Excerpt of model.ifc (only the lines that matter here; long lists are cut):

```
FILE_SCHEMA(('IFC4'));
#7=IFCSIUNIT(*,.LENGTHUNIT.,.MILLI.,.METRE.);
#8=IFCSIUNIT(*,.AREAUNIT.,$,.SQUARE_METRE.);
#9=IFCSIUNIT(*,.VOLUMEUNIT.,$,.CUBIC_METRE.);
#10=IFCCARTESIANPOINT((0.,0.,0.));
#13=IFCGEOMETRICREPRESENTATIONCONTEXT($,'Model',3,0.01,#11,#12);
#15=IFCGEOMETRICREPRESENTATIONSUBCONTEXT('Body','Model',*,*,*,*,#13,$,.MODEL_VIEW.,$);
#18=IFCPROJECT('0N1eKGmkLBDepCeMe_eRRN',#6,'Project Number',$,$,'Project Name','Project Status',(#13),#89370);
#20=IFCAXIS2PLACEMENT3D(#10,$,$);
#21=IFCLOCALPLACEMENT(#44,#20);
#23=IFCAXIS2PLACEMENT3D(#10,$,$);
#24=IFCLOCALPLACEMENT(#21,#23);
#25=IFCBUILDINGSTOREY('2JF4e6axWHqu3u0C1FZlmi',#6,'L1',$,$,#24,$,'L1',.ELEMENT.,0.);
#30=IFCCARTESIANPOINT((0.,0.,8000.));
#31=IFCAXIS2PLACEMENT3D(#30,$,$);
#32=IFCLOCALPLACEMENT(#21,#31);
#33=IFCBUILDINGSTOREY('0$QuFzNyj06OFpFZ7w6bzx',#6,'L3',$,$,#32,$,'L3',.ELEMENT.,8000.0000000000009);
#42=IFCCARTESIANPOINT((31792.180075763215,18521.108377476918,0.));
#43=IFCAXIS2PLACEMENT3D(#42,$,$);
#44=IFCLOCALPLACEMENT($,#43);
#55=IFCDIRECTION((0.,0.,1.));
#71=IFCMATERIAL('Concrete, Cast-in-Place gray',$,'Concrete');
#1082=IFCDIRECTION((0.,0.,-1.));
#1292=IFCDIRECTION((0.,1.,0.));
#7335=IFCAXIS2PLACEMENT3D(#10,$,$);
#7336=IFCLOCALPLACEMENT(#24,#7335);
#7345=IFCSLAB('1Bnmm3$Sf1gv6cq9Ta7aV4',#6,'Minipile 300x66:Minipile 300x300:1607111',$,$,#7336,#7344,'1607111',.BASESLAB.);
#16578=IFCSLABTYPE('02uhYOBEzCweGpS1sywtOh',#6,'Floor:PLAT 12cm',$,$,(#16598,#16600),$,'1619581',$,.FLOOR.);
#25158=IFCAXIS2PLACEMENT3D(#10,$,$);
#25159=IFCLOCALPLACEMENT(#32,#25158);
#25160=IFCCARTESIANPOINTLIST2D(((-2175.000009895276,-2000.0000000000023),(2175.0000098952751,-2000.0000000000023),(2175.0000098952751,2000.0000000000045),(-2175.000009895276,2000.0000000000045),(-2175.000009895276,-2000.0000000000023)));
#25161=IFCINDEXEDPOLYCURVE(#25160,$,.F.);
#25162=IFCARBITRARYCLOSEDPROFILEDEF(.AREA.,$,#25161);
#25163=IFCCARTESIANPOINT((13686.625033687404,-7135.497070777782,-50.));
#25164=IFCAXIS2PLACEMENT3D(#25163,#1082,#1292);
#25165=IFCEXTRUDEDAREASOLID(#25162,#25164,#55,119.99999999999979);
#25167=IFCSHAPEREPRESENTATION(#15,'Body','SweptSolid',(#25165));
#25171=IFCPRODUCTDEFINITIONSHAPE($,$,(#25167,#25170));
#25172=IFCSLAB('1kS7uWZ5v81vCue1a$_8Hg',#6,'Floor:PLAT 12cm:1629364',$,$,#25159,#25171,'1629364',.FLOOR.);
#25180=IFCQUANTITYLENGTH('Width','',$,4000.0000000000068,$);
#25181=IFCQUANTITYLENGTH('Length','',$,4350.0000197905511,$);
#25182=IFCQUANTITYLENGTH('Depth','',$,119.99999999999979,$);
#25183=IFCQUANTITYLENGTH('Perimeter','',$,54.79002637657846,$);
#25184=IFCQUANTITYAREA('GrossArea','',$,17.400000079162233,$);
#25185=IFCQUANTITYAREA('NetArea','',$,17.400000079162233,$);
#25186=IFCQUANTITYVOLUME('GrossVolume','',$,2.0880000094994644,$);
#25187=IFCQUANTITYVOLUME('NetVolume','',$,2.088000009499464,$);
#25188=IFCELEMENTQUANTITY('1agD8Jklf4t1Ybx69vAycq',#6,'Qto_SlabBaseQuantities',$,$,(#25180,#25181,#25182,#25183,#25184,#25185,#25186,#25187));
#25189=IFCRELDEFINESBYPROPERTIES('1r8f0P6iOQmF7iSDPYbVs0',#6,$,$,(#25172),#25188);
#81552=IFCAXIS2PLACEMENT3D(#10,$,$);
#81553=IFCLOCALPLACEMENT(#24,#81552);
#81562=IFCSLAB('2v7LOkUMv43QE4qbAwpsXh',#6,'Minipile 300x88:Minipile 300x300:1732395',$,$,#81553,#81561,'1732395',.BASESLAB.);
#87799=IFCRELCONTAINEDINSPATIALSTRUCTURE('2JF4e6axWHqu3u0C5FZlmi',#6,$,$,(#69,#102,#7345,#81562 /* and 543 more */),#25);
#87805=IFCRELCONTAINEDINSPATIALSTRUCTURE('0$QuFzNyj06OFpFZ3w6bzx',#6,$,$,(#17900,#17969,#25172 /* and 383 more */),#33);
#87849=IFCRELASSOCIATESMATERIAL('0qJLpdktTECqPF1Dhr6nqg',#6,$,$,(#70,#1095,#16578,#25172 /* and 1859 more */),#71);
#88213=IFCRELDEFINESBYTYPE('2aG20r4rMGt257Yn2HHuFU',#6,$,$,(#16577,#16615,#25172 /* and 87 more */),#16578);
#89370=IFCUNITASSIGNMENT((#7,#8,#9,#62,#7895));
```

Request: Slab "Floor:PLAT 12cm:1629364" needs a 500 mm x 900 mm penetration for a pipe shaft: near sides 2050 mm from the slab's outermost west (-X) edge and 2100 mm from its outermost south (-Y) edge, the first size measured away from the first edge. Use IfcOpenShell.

```python
import numpy as np
import ifcopenshell
import ifcopenshell.api.feature
import ifcopenshell.api.geometry
import ifcopenshell.api.pset
import ifcopenshell.api.root
import ifcopenshell.geom
import ifcopenshell.util.element
import ifcopenshell.util.placement
import ifcopenshell.util.representation
import ifcopenshell.util.shape
import ifcopenshell.util.unit

model = ifcopenshell.open("model.ifc")
unit_scale = ifcopenshell.util.unit.calculate_unit_scale(model)
area_scale = ifcopenshell.util.unit.calculate_unit_scale(model, "AREAUNIT")
volume_scale = ifcopenshell.util.unit.calculate_unit_scale(model, "VOLUMEUNIT")
settings = ifcopenshell.geom.settings()


def volume(element):
    """Net volume in cubic metres, openings subtracted."""
    shape = ifcopenshell.geom.create_shape(settings, element)
    return ifcopenshell.util.shape.get_volume(shape.geometry)


slab = model.by_guid("1kS7uWZ5v81vCue1a$_8Hg")
before = volume(slab)

# Extent in the slab's own axes, in metres. The edges named are its -X and -Y sides.
slab_shape = ifcopenshell.geom.create_shape(settings, slab)
vertices = ifcopenshell.util.shape.get_vertices(slab_shape.geometry)
x_min, y_min, bottom = vertices.min(axis=0)
top = vertices[:, 2].max()

opening = ifcopenshell.api.root.create_entity(model, ifc_class="IfcOpeningElement", name="Pipe shaft opening", predefined_type="OPENING")
context = ifcopenshell.util.representation.get_context(model, "Model", "Body", "MODEL_VIEW")
width, depth = 0.5, 0.9
outline = [(0.0, 0.0), (width, 0.0), (width, depth), (0.0, depth), (0.0, 0.0)]
# Overshoot both faces by 50 mm so the cut is clean.
shape = ifcopenshell.api.geometry.add_slab_representation(
    model, context=context, depth=top - bottom + 0.1, polyline=outline
)
ifcopenshell.api.geometry.assign_representation(model, product=opening, representation=shape)

matrix = ifcopenshell.util.placement.get_local_placement(slab.ObjectPlacement)
matrix[:, 3] = matrix @ np.append(np.array([x_min + 2.05, y_min + 2.1, bottom - 0.05]) / unit_scale, 1.0)
ifcopenshell.api.geometry.edit_object_placement(model, product=opening, matrix=matrix, is_si=False)
ifcopenshell.api.feature.add_feature(model, feature=opening, element=slab)

after = volume(slab)

# Update the slab's stored quantities.
qto = model.by_id(ifcopenshell.util.element.get_pset(slab, "Qto_SlabBaseQuantities", should_inherit=False)["id"])
ifcopenshell.api.pset.edit_qto(model, qto=qto, properties={
    "NetArea": after / (top - bottom) / area_scale,
    "NetVolume": after / volume_scale,
})

print(f"slab volume {before:.3f} -> {after:.3f} m3")

model.write("model_updated.ifc")
```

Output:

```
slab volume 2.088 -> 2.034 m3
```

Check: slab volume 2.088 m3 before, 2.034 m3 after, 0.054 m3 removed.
